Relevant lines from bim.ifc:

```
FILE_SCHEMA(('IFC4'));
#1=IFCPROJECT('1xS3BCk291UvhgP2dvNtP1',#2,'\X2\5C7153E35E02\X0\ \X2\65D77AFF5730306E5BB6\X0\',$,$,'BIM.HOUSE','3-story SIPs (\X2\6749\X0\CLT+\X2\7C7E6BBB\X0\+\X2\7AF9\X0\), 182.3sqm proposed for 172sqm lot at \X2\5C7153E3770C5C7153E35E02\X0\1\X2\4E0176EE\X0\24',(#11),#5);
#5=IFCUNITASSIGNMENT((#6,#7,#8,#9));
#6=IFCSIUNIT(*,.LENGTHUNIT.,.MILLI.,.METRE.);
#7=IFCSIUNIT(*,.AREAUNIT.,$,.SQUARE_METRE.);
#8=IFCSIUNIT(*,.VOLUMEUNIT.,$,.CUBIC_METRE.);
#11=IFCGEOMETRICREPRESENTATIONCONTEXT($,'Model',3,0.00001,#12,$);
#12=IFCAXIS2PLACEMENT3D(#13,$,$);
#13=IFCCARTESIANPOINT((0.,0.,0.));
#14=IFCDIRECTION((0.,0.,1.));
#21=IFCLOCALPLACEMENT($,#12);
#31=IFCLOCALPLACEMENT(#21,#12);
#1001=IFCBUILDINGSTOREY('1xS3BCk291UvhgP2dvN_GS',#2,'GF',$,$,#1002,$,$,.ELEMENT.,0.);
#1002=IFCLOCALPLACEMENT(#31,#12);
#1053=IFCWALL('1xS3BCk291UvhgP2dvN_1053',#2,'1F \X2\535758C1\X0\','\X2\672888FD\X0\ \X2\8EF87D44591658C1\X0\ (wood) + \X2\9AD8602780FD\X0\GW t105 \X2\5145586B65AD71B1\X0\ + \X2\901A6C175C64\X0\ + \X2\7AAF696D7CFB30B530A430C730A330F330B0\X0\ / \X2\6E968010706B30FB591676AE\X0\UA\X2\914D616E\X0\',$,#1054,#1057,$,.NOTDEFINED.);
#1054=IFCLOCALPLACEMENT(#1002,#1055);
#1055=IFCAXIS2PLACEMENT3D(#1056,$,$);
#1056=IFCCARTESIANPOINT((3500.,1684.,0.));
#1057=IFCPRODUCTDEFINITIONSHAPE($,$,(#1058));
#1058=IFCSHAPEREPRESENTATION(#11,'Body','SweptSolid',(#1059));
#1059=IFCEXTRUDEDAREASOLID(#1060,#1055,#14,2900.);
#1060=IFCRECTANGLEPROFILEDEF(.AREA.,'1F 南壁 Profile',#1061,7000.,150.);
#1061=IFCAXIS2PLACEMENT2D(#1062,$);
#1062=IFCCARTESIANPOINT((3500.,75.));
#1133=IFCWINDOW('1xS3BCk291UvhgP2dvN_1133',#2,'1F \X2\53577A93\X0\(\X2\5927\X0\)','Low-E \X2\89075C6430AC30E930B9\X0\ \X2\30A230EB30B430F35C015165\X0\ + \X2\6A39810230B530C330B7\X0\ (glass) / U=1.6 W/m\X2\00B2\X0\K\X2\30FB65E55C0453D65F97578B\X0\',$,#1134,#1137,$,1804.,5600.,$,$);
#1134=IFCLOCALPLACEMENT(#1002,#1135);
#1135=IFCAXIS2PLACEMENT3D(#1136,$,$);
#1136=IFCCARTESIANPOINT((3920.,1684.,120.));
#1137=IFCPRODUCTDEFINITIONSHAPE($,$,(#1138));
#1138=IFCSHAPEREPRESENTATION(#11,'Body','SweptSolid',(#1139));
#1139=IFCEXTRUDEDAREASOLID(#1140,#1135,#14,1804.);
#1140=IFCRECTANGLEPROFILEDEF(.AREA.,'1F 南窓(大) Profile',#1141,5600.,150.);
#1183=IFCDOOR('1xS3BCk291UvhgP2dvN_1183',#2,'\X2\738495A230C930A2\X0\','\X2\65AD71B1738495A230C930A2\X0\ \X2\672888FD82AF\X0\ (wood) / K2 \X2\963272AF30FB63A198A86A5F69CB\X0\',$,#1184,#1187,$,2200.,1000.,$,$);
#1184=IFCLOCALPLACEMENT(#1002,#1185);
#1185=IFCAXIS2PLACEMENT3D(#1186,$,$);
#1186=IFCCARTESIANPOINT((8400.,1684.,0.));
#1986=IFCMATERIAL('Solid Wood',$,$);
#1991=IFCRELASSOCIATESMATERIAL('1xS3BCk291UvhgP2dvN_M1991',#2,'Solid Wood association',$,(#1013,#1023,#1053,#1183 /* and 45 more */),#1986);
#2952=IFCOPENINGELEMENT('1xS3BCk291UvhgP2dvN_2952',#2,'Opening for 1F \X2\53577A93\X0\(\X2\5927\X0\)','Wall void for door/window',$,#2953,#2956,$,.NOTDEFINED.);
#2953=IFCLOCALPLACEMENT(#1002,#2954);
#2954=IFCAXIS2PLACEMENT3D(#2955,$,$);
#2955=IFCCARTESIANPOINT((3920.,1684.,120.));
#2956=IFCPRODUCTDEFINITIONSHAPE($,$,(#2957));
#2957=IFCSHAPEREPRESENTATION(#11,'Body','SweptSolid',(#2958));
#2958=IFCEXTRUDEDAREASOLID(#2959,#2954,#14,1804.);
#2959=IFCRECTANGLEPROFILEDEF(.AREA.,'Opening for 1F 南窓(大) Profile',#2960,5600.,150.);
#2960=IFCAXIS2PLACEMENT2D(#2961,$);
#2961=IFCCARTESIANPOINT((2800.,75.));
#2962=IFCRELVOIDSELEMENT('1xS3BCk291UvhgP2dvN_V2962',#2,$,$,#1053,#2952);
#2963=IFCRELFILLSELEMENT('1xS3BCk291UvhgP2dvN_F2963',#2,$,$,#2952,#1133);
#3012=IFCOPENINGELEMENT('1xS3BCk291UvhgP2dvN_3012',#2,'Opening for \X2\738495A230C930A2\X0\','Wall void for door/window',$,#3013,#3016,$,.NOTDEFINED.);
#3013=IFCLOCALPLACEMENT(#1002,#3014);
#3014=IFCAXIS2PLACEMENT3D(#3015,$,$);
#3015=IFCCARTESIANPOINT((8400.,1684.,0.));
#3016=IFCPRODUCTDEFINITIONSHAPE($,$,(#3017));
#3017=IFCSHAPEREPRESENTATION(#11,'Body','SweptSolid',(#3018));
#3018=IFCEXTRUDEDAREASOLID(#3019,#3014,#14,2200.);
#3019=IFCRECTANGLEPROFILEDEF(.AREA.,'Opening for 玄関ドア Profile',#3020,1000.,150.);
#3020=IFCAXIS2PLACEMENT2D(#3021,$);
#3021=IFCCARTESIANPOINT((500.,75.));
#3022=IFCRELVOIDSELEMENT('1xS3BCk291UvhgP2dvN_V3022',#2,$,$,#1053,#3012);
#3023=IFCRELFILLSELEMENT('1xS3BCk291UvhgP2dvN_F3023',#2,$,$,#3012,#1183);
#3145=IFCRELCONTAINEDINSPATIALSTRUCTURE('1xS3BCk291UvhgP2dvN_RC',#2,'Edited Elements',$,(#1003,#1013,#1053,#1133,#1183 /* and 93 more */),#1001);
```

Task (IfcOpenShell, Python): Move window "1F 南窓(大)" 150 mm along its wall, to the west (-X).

```python
import ifcopenshell
import ifcopenshell.api.geometry
import ifcopenshell.util.placement

model = ifcopenshell.open("bim.ifc")

window = model.by_id(1133)
opening = window.FillsVoids[0].RelatingOpeningElement
wall = opening.VoidsElements[0].RelatingBuildingElement

wall_matrix = ifcopenshell.util.placement.get_local_placement(wall.ObjectPlacement)
shift = wall_matrix[:3, 0] * -150.0
before = ifcopenshell.util.placement.get_local_placement(window.ObjectPlacement)[:3, 3].copy()

# The window is not placed relative to its opening, so move both.
for product in (opening, window):
    matrix = ifcopenshell.util.placement.get_local_placement(product.ObjectPlacement)
    matrix[:3, 3] += shift
    ifcopenshell.api.geometry.edit_object_placement(model, product=product, matrix=matrix, is_si=False)

after = ifcopenshell.util.placement.get_local_placement(window.ObjectPlacement)[:3, 3]
print("window moved by", (after - before).round(3) + 0.0)

model.write("bim_v2.ifc")
```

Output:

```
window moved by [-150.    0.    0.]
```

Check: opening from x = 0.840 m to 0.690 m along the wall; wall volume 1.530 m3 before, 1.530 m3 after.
